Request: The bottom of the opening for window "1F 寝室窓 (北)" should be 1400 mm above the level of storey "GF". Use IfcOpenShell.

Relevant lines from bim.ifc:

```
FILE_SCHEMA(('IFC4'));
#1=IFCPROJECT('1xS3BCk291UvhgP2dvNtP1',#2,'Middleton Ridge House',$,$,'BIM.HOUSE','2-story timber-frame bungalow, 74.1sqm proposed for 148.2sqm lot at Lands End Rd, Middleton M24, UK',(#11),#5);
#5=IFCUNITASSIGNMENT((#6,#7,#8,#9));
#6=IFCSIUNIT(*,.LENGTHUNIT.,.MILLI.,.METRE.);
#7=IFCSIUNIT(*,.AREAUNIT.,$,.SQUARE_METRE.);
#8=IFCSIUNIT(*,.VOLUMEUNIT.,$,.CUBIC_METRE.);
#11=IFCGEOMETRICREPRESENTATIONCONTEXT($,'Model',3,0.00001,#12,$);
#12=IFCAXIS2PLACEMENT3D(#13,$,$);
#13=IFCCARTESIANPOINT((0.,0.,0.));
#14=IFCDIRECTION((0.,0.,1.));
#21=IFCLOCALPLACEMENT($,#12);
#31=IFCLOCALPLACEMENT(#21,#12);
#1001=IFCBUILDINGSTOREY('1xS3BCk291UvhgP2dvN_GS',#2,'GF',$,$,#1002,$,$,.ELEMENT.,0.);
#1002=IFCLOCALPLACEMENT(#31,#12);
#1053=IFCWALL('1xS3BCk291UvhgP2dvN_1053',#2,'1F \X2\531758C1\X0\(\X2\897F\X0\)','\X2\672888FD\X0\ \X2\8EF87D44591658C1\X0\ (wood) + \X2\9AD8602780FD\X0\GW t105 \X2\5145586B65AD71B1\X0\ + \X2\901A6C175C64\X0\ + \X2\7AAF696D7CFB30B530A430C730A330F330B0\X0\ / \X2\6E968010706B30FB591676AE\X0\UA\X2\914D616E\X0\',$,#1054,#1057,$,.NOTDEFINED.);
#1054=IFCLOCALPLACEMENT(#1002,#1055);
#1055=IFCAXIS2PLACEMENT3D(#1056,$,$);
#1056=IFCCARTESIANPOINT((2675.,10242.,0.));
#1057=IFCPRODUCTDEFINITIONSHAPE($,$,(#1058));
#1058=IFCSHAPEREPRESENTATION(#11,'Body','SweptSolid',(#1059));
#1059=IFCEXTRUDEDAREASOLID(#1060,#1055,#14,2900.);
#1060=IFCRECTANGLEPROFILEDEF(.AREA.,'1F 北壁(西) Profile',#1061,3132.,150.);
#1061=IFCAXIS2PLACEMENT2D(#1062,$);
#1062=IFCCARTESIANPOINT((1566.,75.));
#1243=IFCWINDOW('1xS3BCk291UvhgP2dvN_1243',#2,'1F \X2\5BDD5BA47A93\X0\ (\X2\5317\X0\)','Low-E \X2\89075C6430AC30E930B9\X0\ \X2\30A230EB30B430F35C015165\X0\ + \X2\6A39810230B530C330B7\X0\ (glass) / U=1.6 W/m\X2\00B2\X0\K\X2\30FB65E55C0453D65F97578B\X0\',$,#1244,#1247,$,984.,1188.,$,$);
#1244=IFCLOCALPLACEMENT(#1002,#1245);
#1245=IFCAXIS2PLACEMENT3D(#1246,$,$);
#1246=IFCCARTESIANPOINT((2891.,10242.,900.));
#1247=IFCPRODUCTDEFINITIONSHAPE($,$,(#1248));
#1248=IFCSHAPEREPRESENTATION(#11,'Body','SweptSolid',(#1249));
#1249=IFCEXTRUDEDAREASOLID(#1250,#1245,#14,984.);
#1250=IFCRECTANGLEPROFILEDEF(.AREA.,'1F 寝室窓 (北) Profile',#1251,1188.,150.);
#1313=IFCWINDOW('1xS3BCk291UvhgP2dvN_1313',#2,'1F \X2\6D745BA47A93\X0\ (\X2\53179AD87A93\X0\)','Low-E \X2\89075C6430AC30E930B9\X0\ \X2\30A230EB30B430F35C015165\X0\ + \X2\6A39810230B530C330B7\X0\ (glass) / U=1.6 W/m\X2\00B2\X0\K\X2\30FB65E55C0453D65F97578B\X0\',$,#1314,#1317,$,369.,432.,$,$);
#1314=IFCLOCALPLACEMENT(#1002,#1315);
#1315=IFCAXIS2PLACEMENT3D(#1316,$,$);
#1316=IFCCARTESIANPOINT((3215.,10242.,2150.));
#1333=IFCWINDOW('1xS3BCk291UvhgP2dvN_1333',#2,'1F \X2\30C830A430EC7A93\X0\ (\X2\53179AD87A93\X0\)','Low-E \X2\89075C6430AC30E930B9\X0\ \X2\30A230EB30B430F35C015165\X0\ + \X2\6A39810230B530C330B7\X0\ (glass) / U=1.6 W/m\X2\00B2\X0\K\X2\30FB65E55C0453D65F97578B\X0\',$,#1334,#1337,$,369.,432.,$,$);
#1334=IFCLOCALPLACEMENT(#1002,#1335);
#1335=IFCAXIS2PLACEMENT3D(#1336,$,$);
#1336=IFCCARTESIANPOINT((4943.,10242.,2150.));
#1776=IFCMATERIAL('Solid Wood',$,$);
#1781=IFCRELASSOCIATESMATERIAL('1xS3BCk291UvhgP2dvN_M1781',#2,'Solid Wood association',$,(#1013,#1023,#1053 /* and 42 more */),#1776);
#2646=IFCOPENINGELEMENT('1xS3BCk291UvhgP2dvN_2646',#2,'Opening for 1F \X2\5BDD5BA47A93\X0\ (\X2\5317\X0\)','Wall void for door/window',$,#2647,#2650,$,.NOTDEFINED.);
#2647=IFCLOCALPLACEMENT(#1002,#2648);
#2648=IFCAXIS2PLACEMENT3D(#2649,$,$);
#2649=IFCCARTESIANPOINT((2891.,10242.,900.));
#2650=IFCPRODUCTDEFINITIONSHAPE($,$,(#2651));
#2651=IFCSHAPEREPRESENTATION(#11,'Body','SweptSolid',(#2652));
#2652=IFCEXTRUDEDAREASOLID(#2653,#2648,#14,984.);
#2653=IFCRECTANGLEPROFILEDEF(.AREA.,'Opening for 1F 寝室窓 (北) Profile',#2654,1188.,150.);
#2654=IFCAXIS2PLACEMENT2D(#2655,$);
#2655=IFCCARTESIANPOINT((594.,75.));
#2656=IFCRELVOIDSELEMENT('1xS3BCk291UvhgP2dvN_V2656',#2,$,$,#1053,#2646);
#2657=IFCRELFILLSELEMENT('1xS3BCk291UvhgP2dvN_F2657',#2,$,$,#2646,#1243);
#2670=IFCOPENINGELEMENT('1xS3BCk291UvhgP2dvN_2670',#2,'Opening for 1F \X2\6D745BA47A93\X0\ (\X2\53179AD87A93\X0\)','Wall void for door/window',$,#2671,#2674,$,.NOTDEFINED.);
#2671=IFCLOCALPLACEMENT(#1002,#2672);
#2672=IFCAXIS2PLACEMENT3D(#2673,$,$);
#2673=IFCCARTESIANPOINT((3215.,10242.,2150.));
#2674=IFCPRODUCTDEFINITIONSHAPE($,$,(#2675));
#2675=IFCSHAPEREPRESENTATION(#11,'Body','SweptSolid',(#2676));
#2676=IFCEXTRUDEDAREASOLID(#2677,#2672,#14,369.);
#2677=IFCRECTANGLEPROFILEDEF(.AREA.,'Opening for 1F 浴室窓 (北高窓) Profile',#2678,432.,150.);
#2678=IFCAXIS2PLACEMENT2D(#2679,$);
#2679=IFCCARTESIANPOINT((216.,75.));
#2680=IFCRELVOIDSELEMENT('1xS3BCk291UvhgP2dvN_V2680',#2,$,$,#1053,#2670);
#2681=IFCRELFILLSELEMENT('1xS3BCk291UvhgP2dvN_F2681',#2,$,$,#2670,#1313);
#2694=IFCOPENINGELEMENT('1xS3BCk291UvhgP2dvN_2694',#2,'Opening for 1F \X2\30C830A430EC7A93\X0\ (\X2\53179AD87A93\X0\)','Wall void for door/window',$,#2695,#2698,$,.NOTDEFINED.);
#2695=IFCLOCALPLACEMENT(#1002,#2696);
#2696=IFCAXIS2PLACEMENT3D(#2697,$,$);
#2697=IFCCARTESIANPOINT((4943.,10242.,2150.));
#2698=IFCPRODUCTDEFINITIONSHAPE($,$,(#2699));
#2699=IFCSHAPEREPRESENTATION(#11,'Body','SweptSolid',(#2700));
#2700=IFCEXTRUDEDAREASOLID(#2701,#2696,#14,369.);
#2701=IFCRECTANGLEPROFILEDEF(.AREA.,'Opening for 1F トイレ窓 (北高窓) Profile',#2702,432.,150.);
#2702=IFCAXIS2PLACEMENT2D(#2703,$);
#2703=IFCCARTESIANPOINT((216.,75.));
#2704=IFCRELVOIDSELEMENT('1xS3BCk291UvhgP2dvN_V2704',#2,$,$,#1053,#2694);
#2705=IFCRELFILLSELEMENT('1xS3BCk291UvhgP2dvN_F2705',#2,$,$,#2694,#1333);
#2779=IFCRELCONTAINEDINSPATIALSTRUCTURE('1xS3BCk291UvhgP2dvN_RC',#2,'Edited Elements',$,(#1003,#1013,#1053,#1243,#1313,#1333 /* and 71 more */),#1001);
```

```python
import numpy as np
import ifcopenshell
import ifcopenshell.api.geometry
import ifcopenshell.geom
import ifcopenshell.util.element
import ifcopenshell.util.placement
import ifcopenshell.util.shape
import ifcopenshell.util.unit

model = ifcopenshell.open("bim.ifc")
unit_scale = ifcopenshell.util.unit.calculate_unit_scale(model)

window = model.by_guid("1xS3BCk291UvhgP2dvN_1243")
opening = window.FillsVoids[0].RelatingOpeningElement
storey = ifcopenshell.util.element.get_container(window, ifc_class="IfcBuildingStorey")
level = ifcopenshell.util.placement.get_local_placement(storey.ObjectPlacement)[2, 3]

# The opening's origin need not be at the sill, so measure its lowest point.
shape = ifcopenshell.geom.create_shape(ifcopenshell.geom.settings(), opening)
bottom = ifcopenshell.util.shape.get_shape_bottom_elevation(shape, shape.geometry) / unit_scale
dz = level + 1.4 / unit_scale - bottom

shift = np.array([0.0, 0.0, dz])
# The window is not placed relative to its opening, so move both.
for product in (opening, window):
    matrix = ifcopenshell.util.placement.get_local_placement(product.ObjectPlacement)
    matrix[:3, 3] += shift
    ifcopenshell.api.geometry.edit_object_placement(model, product=product, matrix=matrix, is_si=False)

print(f"moved by {dz * unit_scale:+.3f} m")

model.write("bim_updated.ifc")
```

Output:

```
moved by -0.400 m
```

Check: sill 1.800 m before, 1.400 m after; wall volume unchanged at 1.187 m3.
